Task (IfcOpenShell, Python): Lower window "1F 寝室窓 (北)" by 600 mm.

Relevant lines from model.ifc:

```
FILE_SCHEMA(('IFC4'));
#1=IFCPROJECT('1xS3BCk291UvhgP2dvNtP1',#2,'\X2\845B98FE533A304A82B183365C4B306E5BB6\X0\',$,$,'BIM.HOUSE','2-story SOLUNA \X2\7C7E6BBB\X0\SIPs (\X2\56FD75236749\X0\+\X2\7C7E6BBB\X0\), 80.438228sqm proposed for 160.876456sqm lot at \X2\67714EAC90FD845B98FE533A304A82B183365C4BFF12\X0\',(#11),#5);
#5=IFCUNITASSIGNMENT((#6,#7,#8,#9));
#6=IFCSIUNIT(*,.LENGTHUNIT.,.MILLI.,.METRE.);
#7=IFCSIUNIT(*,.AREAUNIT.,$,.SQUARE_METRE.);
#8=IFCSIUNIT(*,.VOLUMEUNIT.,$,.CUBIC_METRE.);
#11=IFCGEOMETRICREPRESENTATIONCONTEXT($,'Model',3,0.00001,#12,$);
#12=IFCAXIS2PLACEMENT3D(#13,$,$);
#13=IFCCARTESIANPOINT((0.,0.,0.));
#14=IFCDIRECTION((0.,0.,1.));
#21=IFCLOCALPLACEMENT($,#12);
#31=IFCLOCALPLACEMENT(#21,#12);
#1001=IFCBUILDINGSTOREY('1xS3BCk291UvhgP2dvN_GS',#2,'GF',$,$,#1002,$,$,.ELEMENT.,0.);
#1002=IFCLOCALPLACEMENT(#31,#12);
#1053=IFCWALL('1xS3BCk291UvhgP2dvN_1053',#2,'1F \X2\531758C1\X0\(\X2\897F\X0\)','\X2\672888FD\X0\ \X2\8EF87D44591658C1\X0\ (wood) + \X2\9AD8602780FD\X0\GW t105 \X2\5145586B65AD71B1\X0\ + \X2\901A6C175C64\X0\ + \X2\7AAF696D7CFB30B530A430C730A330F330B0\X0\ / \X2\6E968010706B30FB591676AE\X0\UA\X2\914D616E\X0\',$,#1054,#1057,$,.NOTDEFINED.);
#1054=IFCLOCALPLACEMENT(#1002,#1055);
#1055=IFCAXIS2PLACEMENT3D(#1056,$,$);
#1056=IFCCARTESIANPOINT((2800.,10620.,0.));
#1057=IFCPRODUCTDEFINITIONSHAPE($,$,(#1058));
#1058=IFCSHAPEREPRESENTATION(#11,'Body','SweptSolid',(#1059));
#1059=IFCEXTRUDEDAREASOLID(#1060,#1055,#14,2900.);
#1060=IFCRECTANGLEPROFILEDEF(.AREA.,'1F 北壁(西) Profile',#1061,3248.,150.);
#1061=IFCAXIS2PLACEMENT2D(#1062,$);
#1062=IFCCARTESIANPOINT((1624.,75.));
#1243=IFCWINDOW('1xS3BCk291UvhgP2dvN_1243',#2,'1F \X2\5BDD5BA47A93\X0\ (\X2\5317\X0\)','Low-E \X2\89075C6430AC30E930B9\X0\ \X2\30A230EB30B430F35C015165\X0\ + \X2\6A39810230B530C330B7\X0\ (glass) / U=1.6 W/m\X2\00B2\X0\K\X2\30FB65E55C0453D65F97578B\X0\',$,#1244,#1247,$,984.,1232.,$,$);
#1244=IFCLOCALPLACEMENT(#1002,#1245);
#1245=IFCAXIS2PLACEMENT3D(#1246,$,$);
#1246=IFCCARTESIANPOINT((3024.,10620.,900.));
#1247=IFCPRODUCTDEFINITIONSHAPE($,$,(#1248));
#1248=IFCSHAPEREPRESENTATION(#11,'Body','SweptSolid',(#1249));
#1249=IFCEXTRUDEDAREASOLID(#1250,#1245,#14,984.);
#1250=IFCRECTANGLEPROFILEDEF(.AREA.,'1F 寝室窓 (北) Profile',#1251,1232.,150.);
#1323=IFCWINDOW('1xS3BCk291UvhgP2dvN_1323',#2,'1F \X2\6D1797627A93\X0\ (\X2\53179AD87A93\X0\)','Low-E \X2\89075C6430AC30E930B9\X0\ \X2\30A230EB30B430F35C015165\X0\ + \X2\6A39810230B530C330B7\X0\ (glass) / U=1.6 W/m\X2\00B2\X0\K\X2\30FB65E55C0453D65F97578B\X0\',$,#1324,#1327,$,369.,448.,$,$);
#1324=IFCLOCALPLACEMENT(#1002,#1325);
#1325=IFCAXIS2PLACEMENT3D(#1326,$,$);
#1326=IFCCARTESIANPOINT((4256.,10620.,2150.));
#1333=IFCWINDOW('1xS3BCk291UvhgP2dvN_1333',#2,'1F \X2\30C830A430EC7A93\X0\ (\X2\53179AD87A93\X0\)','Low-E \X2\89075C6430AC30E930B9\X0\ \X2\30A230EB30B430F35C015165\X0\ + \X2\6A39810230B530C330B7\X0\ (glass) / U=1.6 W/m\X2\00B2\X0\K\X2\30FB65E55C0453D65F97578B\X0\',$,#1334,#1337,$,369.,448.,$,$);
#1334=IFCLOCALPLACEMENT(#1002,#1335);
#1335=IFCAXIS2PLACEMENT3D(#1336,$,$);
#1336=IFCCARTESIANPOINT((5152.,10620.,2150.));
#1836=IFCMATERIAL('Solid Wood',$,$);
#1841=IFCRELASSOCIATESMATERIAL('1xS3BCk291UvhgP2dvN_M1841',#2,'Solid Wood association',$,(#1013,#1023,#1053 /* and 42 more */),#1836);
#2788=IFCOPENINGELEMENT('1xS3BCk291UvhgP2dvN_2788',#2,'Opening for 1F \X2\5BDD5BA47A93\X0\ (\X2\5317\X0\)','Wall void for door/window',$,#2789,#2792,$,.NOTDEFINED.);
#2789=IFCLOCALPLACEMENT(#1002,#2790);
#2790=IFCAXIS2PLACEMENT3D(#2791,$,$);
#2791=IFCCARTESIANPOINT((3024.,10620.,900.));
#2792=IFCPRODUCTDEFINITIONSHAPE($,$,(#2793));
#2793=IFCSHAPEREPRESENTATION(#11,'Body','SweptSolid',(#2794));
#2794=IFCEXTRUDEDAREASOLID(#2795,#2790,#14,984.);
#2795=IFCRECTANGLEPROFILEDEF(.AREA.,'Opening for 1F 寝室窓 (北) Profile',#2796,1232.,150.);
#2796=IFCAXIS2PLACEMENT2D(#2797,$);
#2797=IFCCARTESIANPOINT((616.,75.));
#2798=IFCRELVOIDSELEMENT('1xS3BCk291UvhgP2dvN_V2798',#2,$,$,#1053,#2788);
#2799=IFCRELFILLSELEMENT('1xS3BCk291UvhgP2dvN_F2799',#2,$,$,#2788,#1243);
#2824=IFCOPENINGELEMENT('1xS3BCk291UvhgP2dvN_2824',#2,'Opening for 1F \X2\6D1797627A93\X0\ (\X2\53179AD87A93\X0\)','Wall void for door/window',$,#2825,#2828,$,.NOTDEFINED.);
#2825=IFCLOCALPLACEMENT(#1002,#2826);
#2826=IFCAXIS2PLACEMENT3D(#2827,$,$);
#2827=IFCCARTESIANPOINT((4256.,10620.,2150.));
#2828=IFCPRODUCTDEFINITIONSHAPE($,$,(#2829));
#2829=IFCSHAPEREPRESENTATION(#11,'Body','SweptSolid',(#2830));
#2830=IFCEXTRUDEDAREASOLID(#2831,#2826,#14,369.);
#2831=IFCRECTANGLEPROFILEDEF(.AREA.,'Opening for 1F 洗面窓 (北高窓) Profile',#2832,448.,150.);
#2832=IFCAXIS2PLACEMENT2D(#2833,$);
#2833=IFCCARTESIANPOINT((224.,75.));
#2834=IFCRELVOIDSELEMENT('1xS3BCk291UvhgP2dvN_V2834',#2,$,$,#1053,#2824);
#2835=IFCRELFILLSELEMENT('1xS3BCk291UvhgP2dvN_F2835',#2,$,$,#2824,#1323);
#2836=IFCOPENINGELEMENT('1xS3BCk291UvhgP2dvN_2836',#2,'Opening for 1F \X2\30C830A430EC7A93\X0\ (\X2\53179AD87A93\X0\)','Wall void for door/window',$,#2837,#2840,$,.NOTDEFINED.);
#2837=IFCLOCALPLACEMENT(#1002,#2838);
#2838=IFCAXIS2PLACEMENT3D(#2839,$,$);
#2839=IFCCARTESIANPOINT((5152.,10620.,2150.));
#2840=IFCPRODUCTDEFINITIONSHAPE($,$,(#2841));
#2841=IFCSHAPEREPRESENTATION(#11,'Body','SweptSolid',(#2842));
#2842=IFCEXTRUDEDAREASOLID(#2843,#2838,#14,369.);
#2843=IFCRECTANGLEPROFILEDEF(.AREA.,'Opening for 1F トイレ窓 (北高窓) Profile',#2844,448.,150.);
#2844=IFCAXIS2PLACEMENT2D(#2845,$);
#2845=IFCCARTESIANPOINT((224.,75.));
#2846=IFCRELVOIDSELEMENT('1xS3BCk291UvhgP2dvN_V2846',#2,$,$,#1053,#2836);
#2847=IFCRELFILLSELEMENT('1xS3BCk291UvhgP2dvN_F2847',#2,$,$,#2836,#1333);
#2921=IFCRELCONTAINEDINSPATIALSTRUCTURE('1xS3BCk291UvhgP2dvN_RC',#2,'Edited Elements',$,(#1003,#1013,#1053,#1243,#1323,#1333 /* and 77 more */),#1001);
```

```python
import numpy as np
import ifcopenshell
import ifcopenshell.api.geometry
import ifcopenshell.util.placement
import ifcopenshell.util.unit

model = ifcopenshell.open("model.ifc")
unit_scale = ifcopenshell.util.unit.calculate_unit_scale(model)

window = model.by_guid("1xS3BCk291UvhgP2dvN_1243")
opening = window.FillsVoids[0].RelatingOpeningElement
dz = -600.0

shift = np.array([0.0, 0.0, dz])
# The window is not placed relative to its opening, so move both.
for product in (opening, window):
    matrix = ifcopenshell.util.placement.get_local_placement(product.ObjectPlacement)
    matrix[:3, 3] += shift
    ifcopenshell.api.geometry.edit_object_placement(model, product=product, matrix=matrix, is_si=False)

print(f"moved by {dz * unit_scale:+.3f} m")

model.write("model_rev.ifc")
```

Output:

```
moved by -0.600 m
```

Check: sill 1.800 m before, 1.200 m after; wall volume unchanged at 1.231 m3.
